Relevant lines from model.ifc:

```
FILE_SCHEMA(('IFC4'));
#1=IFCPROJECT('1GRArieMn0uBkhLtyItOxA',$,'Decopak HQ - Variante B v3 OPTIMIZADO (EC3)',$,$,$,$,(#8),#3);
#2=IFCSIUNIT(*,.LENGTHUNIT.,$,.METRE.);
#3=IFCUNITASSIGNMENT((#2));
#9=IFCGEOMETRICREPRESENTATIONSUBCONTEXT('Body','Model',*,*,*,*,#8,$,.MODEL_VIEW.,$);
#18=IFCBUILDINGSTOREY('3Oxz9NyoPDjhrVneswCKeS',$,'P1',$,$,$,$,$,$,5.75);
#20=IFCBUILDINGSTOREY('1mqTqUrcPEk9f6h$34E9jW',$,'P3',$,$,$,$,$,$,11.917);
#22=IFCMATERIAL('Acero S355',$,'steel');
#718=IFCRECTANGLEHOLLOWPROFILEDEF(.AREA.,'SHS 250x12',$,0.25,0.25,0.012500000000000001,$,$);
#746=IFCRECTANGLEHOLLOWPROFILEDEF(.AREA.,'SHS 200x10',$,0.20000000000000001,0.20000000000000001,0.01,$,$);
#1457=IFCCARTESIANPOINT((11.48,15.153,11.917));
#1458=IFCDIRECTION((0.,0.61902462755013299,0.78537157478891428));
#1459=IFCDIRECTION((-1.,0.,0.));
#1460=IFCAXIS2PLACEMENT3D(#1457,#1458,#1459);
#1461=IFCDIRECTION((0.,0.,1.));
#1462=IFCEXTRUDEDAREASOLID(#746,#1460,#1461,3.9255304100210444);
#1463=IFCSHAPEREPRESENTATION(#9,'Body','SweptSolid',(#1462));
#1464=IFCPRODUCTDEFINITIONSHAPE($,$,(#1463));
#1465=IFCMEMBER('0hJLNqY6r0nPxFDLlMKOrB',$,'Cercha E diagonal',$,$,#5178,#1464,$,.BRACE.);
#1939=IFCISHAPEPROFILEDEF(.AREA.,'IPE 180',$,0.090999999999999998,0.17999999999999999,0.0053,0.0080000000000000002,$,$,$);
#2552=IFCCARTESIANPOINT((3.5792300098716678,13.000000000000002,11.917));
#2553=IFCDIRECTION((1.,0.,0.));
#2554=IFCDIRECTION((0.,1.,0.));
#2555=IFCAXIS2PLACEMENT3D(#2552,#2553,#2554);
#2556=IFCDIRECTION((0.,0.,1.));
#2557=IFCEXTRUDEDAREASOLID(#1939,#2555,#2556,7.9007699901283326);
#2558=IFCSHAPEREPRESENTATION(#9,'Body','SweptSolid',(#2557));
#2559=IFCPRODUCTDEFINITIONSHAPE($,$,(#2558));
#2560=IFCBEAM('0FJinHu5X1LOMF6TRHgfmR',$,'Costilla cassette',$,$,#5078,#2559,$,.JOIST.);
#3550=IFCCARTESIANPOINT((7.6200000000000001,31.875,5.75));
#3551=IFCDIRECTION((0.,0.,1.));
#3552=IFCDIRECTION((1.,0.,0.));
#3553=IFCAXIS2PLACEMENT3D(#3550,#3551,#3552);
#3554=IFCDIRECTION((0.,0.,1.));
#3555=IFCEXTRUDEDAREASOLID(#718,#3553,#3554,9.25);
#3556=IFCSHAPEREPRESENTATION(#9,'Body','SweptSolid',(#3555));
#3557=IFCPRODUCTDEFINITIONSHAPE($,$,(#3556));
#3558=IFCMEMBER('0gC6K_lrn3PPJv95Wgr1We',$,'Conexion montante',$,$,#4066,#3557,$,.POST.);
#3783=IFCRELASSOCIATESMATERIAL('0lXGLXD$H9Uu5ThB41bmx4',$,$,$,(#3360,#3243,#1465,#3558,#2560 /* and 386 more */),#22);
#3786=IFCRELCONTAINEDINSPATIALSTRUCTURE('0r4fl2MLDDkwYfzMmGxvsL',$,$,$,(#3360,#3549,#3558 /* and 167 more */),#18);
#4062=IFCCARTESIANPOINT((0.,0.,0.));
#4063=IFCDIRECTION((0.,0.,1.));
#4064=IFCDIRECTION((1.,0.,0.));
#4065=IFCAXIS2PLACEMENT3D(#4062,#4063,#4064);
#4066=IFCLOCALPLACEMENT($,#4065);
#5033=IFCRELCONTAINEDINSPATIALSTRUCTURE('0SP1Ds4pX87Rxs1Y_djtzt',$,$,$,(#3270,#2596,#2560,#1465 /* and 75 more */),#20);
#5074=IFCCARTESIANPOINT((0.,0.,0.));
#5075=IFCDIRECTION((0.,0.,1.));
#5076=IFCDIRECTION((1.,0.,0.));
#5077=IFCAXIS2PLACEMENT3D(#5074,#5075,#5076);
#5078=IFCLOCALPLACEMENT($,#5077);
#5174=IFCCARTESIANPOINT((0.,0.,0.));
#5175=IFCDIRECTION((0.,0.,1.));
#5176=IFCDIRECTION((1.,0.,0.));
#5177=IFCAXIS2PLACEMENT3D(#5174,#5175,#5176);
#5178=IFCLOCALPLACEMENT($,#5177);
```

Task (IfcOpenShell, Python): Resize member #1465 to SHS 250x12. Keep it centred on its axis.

```python
import ifcopenshell
import ifcopenshell.util.element
import ifcopenshell.util.representation

model = ifcopenshell.open("model.ifc")

member = model.by_guid("0hJLNqY6r0nPxFDLlMKOrB")
source = next(p for p in model.by_type("IfcRectangleHollowProfileDef") if p.ProfileName == "SHS 250x12")

body = ifcopenshell.util.representation.get_representation(member, "Model", "Body")
solid = body.Items[0]
old_profile = solid.SweptArea

# Copy the section's sizes but keep this member's own profile position.
profile = ifcopenshell.util.element.copy(model, source)
profile.Position = old_profile.Position
solid.SweptArea = profile
if not model.get_total_inverses(old_profile):
    ifcopenshell.util.element.remove_deep2(model, old_profile)

print(solid.SweptArea)

model.write("model_rev.ifc")
```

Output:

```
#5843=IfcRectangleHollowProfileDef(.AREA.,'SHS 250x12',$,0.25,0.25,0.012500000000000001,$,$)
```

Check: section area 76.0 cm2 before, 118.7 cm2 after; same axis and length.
